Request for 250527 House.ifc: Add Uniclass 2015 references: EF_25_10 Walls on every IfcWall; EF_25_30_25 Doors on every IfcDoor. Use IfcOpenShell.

First a look at what the model holds.

```python
import ifcopenshell

model = ifcopenshell.open("250527 House.ifc")
print(model.schema)
print("classifications:", [c.Name for c in model.by_type("IfcClassification")])
for ifc_class in ("IfcDoor", "IfcRoof", "IfcStair", "IfcWall", "IfcWindow"):
    print(ifc_class, len(model.by_type(ifc_class)))
```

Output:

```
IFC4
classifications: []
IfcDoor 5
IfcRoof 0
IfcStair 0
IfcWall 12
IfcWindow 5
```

```python
import ifcopenshell
import ifcopenshell.api.classification

model = ifcopenshell.open("250527 House.ifc")

system = ifcopenshell.api.classification.add_classification(model, classification="Uniclass 2015")

codes = {
    "IfcWall": ("EF_25_10", "Walls"),
    "IfcDoor": ("EF_25_30_25", "Doors"),
}
for ifc_class, (code, name) in codes.items():
    products = model.by_type(ifc_class)
    ifcopenshell.api.classification.add_reference(
        model, products=products, classification=system, identification=code, name=name
    )
    print(code, len(products))

model.write("250527 House_rev.ifc")
```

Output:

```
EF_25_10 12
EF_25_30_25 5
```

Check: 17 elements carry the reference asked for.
